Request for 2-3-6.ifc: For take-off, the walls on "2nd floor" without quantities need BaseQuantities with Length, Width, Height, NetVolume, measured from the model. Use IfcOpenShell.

First a look at what the model holds.

```python
import ifcopenshell
import ifcopenshell.util.element
import ifcopenshell.util.unit

model = ifcopenshell.open("2-3-6.ifc")
print(model.schema)
for unit_type in ("LENGTHUNIT", "AREAUNIT", "VOLUMEUNIT"):
    print(unit_type, ifcopenshell.util.unit.calculate_unit_scale(model, unit_type))
storey = next(s for s in model.by_type("IfcBuildingStorey") if s.Name == "2nd floor")
walls = [e for e in ifcopenshell.util.element.get_decomposition(storey) if e.is_a("IfcWall")]
for e in sorted(walls, key=lambda e: e.id()):
    print(e.id(), e.is_a(), e.Name, list(ifcopenshell.util.element.get_psets(e, qtos_only=True)), sep=" | ")
```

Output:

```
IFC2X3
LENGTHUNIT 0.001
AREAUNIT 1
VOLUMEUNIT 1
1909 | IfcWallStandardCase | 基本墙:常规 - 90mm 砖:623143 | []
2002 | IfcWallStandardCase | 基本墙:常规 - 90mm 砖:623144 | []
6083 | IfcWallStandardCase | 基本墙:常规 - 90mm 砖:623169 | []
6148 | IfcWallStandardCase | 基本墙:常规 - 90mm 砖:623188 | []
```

```python
import ifcopenshell
import ifcopenshell.api.pset
import ifcopenshell.geom
import ifcopenshell.util.element
import ifcopenshell.util.shape
import ifcopenshell.util.unit

model = ifcopenshell.open("2-3-6.ifc")
unit_scale = ifcopenshell.util.unit.calculate_unit_scale(model)
volume_scale = ifcopenshell.util.unit.calculate_unit_scale(model, "VOLUMEUNIT")
settings = ifcopenshell.geom.settings()

storey = next(s for s in model.by_type("IfcBuildingStorey") if s.Name == "2nd floor")
walls = [e for e in ifcopenshell.util.element.get_decomposition(storey) if e.is_a("IfcWall")]

for e in sorted(walls, key=lambda e: e.id()):
    if ifcopenshell.util.element.get_psets(e, qtos_only=True, should_inherit=False):
        continue
    # Geometry comes back in metres, in the element's own axes.
    shape = ifcopenshell.geom.create_shape(settings, e)
    values = {
        "Length": ifcopenshell.util.shape.get_x(shape.geometry) / unit_scale,
        "Width": ifcopenshell.util.shape.get_y(shape.geometry) / unit_scale,
        "Height": ifcopenshell.util.shape.get_z(shape.geometry) / unit_scale,
        "NetVolume": ifcopenshell.util.shape.get_volume(shape.geometry) / volume_scale,
    }
    qto = ifcopenshell.api.pset.add_qto(model, product=e, name="BaseQuantities")
    ifcopenshell.api.pset.edit_qto(model, qto=qto, properties=values)
    print(e.id(), {k: round(v, 3) for k, v in values.items()})

model.write("2-3-6_edited.ifc")
```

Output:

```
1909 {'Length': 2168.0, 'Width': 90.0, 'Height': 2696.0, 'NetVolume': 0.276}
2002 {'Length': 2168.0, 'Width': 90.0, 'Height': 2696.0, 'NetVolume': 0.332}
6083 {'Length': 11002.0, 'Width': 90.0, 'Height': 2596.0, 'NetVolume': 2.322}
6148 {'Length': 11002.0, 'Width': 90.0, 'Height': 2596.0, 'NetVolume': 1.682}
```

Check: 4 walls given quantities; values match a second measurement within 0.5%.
